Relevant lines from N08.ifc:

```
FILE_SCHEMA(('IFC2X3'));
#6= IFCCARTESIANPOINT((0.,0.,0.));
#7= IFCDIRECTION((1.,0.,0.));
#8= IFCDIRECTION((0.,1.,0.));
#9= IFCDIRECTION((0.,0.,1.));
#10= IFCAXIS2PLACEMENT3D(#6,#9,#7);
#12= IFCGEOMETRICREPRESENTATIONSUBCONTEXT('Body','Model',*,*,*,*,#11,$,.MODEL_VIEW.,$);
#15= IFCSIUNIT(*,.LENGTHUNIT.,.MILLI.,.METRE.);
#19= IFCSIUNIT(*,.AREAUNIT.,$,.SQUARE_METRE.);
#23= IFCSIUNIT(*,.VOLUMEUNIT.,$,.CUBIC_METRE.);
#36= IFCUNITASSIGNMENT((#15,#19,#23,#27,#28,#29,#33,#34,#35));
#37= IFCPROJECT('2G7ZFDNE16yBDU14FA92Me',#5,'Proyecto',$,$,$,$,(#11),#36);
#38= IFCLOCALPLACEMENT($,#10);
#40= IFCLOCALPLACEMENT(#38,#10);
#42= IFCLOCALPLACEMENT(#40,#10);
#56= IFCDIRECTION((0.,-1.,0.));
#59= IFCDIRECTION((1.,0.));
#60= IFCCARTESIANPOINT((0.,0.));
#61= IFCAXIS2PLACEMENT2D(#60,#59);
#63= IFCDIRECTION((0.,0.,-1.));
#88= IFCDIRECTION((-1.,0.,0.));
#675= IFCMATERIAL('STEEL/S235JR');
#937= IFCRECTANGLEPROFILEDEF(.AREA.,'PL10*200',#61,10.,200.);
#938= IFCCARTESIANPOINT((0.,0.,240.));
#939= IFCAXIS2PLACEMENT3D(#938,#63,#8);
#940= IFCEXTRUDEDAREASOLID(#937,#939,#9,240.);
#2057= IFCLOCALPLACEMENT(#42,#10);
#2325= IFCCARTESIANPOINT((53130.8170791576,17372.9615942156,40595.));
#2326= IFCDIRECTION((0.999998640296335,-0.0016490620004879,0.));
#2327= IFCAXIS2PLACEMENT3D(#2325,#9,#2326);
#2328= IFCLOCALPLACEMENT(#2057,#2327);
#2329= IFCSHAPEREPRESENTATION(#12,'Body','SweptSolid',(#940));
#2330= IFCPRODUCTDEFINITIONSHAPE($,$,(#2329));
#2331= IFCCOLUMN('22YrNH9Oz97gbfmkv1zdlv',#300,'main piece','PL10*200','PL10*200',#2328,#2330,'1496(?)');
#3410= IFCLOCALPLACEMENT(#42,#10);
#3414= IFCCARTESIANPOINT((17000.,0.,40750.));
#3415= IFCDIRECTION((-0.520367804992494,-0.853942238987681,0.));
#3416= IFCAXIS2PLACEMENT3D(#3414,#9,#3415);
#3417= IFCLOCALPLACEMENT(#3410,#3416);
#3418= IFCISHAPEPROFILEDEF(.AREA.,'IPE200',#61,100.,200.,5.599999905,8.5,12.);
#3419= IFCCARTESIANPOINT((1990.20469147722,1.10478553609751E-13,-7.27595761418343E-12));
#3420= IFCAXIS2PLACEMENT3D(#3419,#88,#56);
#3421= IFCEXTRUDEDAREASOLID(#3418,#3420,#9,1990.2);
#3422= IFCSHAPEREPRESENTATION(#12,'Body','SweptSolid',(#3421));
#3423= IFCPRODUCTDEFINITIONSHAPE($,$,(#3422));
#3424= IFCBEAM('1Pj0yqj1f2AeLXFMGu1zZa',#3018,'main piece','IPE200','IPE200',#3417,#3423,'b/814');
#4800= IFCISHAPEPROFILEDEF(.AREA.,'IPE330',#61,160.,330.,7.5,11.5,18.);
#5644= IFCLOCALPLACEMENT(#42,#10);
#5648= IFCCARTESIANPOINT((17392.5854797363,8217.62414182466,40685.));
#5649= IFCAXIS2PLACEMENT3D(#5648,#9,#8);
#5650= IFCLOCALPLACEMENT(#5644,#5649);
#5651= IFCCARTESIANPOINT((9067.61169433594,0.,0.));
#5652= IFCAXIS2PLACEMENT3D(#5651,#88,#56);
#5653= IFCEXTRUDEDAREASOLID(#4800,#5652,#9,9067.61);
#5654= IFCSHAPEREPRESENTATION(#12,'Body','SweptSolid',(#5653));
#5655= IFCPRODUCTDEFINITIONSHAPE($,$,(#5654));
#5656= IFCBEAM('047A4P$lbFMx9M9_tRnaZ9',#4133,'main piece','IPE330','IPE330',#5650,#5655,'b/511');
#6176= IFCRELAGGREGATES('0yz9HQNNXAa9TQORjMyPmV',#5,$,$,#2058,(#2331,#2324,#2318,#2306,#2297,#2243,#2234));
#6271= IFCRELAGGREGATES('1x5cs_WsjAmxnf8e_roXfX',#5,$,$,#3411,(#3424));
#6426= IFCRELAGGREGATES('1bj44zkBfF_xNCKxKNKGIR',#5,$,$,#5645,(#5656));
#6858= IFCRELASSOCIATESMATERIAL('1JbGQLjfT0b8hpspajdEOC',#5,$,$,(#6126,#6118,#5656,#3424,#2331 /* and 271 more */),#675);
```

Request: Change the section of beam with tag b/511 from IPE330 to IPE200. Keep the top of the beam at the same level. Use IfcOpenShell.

```python
import ifcopenshell
import ifcopenshell.util.element
import ifcopenshell.util.representation

model = ifcopenshell.open("N08.ifc")

member = model.by_guid("047A4P$lbFMx9M9_tRnaZ9")
source = next(p for p in model.by_type("IfcIShapeProfileDef") if p.ProfileName == "IPE200")

body = ifcopenshell.util.representation.get_representation(member, "Model", "Body")
solid = body.Items[0]
old_profile = solid.SweptArea

# Copy the section's sizes but keep this member's own profile position.
profile = ifcopenshell.util.element.copy(model, source)
# Profiles are centred, so shift by half the change in depth to hold the top.
shift = (old_profile.OverallDepth - profile.OverallDepth) / 2
x, y = old_profile.Position.Location.Coordinates
up = (0.0, 1.0)  # upwards, in the solid's own plane
location = model.createIfcCartesianPoint((x + up[0] * shift, y + up[1] * shift))
profile.Position = model.createIfcAxis2Placement2D(location, old_profile.Position.RefDirection)
solid.SweptArea = profile
if not model.get_total_inverses(old_profile):
    ifcopenshell.util.element.remove_deep2(model, old_profile)
member.Description = member.Description.replace("IPE330", "IPE200")
member.ObjectType = member.ObjectType.replace("IPE330", "IPE200")

print(solid.SweptArea)

model.write("N08_edited.ifc")
```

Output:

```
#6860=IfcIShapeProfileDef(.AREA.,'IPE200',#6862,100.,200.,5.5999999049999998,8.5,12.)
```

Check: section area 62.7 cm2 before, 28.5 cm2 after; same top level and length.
